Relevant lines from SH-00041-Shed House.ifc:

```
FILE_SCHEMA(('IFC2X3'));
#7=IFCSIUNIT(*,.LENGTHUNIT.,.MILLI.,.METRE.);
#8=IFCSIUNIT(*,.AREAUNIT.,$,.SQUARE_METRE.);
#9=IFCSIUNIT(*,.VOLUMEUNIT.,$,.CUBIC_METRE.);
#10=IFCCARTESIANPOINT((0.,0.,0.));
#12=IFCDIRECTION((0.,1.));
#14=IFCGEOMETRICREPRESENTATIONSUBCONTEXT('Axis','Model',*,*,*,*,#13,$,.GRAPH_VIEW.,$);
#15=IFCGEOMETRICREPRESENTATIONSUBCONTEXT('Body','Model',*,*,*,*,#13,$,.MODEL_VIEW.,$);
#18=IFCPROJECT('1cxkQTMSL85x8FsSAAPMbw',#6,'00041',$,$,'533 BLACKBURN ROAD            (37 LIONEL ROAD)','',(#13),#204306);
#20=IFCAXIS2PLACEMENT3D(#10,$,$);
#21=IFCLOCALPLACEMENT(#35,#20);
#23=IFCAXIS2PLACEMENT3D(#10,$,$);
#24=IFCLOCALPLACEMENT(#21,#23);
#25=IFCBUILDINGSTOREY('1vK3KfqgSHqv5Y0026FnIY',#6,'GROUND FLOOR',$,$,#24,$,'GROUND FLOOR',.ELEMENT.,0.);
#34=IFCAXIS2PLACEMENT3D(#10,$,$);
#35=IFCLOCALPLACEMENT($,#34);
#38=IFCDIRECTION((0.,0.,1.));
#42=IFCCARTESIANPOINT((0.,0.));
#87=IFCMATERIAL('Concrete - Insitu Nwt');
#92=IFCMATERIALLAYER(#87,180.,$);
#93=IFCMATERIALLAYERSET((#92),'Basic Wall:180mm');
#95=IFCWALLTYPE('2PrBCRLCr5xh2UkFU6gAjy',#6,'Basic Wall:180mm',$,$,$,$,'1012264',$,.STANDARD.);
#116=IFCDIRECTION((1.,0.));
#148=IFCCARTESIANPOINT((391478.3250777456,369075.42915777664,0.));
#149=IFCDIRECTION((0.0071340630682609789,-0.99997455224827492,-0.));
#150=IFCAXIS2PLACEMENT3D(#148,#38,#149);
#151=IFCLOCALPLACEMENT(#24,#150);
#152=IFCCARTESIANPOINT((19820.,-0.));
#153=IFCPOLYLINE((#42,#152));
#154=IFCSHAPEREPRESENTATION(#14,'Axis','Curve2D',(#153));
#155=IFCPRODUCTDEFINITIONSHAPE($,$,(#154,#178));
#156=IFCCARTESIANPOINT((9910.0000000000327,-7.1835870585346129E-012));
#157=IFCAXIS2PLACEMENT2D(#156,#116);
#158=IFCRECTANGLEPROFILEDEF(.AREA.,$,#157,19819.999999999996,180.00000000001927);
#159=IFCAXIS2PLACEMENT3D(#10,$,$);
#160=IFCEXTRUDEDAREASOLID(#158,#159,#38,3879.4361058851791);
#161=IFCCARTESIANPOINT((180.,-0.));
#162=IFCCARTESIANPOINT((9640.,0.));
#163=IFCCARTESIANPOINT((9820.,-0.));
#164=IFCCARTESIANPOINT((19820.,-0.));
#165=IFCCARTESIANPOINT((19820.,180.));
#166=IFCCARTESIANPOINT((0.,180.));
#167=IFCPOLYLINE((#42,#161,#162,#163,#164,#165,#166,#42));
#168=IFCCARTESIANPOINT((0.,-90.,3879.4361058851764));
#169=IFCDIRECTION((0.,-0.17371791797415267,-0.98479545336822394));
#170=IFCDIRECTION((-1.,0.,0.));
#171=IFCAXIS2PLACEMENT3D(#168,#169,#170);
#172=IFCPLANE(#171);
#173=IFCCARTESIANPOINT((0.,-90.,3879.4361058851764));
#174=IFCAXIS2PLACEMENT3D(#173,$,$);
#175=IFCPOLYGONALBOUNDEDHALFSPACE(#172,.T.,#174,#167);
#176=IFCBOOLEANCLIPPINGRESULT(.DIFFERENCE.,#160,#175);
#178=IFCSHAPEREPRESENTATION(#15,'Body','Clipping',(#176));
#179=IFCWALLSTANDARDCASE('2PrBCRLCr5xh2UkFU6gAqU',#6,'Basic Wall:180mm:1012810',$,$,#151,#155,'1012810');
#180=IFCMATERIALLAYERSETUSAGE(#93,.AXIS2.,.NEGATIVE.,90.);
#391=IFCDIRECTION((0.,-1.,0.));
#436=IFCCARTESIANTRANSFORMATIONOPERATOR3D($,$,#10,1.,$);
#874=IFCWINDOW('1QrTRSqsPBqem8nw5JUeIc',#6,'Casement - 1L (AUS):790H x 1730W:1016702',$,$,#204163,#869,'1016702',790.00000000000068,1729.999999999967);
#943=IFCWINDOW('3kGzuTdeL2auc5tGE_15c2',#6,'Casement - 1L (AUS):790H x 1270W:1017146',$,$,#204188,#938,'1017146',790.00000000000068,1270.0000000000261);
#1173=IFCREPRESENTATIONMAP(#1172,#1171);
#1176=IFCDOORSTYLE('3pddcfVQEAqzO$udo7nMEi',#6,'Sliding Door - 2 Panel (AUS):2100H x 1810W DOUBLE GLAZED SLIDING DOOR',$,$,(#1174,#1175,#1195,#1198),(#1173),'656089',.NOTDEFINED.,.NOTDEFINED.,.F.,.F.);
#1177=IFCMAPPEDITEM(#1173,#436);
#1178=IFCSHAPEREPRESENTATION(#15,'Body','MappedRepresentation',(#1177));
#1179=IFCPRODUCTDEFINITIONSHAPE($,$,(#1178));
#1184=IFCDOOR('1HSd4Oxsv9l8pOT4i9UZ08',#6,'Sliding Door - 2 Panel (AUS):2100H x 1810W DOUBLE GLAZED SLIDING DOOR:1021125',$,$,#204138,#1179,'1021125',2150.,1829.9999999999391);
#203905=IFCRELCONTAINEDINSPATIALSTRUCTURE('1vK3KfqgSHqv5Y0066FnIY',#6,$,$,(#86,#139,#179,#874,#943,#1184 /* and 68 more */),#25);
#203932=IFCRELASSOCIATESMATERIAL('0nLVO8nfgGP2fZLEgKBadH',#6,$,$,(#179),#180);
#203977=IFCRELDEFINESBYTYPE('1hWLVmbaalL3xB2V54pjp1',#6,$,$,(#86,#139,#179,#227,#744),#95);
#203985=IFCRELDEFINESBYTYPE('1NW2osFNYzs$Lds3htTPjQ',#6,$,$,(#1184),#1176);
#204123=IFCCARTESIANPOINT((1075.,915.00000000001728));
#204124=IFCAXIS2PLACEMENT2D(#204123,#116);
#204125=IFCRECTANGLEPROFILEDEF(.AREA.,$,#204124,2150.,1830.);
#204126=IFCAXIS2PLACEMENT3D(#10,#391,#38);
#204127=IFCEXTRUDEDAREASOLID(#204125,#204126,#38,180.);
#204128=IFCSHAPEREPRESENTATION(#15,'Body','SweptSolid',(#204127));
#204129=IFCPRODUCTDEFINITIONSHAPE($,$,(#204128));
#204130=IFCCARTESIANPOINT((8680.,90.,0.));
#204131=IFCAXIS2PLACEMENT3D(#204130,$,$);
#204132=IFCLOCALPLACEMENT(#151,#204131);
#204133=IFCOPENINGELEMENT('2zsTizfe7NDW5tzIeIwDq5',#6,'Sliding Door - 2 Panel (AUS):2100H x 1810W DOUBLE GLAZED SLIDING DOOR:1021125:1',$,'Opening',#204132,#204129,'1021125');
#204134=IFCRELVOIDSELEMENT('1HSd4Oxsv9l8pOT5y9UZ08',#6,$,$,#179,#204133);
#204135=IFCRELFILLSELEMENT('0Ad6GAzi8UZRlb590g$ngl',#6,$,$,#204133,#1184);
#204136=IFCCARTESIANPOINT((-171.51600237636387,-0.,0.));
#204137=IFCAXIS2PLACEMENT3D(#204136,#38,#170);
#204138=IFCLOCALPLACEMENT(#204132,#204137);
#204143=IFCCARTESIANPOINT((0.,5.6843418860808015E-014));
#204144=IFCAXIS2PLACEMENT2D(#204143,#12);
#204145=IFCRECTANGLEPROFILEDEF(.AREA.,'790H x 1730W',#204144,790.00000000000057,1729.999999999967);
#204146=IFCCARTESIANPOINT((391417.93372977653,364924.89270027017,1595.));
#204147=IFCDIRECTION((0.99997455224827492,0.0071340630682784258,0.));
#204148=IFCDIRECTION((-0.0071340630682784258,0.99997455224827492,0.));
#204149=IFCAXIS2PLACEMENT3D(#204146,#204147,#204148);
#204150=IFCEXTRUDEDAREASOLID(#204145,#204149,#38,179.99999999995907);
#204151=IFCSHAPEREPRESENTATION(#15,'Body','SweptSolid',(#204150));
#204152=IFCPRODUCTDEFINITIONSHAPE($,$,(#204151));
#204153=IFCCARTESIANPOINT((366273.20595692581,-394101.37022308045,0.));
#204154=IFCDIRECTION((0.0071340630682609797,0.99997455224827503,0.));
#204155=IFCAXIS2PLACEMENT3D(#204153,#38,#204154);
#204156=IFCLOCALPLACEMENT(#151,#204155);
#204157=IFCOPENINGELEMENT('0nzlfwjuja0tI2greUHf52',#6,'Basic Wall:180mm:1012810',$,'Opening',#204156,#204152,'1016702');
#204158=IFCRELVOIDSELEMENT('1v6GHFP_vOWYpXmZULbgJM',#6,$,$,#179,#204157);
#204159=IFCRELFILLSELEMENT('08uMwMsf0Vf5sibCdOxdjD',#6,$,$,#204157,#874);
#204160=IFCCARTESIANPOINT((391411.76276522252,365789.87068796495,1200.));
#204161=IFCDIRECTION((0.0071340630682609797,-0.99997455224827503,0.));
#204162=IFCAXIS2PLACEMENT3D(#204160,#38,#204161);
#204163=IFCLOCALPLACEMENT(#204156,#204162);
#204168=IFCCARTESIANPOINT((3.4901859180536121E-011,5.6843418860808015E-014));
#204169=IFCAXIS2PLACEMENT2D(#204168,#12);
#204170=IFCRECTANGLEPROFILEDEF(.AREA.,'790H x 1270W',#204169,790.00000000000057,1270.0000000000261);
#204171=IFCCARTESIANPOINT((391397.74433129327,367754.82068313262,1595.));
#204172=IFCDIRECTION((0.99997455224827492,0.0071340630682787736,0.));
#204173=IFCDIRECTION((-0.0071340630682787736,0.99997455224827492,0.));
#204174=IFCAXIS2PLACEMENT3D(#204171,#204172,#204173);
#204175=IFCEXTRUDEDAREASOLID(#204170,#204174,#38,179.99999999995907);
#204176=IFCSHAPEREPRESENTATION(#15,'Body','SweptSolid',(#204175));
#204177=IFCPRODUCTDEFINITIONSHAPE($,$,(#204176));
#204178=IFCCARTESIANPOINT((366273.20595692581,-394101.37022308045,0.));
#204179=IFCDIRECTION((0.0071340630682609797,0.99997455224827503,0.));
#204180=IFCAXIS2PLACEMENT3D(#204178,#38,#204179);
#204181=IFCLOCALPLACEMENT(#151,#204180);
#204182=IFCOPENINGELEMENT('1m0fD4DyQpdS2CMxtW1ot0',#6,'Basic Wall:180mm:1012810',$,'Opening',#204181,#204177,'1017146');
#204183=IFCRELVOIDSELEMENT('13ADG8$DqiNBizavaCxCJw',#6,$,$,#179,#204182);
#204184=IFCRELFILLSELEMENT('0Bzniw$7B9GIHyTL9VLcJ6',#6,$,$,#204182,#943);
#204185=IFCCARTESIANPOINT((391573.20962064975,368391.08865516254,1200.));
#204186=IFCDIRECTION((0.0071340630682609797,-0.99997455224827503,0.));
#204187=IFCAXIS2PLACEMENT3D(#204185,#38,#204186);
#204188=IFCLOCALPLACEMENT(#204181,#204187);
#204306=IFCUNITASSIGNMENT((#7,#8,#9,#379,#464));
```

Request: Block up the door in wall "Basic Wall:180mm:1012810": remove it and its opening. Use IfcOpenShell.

```python
import ifcopenshell
import ifcopenshell.api.feature
import ifcopenshell.api.root
import ifcopenshell.geom
import ifcopenshell.util.shape

model = ifcopenshell.open("SH-00041-Shed House.ifc")
settings = ifcopenshell.geom.settings()


def volume(element):
    """Net volume in cubic metres, openings subtracted."""
    shape = ifcopenshell.geom.create_shape(settings, element)
    return ifcopenshell.util.shape.get_volume(shape.geometry)


door = model.by_guid("1HSd4Oxsv9l8pOT4i9UZ08")
opening = door.FillsVoids[0].RelatingOpeningElement
wall = opening.VoidsElements[0].RelatingBuildingElement
before = volume(wall)

ifcopenshell.api.root.remove_product(model, product=door)
ifcopenshell.api.feature.remove_feature(model, feature=opening)

after = volume(wall)

print(f"wall volume {before:.3f} -> {after:.3f} m3")

model.write("SH-00041-Shed House_rev.ifc")
```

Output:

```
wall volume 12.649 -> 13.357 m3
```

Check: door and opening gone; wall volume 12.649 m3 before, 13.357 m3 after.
